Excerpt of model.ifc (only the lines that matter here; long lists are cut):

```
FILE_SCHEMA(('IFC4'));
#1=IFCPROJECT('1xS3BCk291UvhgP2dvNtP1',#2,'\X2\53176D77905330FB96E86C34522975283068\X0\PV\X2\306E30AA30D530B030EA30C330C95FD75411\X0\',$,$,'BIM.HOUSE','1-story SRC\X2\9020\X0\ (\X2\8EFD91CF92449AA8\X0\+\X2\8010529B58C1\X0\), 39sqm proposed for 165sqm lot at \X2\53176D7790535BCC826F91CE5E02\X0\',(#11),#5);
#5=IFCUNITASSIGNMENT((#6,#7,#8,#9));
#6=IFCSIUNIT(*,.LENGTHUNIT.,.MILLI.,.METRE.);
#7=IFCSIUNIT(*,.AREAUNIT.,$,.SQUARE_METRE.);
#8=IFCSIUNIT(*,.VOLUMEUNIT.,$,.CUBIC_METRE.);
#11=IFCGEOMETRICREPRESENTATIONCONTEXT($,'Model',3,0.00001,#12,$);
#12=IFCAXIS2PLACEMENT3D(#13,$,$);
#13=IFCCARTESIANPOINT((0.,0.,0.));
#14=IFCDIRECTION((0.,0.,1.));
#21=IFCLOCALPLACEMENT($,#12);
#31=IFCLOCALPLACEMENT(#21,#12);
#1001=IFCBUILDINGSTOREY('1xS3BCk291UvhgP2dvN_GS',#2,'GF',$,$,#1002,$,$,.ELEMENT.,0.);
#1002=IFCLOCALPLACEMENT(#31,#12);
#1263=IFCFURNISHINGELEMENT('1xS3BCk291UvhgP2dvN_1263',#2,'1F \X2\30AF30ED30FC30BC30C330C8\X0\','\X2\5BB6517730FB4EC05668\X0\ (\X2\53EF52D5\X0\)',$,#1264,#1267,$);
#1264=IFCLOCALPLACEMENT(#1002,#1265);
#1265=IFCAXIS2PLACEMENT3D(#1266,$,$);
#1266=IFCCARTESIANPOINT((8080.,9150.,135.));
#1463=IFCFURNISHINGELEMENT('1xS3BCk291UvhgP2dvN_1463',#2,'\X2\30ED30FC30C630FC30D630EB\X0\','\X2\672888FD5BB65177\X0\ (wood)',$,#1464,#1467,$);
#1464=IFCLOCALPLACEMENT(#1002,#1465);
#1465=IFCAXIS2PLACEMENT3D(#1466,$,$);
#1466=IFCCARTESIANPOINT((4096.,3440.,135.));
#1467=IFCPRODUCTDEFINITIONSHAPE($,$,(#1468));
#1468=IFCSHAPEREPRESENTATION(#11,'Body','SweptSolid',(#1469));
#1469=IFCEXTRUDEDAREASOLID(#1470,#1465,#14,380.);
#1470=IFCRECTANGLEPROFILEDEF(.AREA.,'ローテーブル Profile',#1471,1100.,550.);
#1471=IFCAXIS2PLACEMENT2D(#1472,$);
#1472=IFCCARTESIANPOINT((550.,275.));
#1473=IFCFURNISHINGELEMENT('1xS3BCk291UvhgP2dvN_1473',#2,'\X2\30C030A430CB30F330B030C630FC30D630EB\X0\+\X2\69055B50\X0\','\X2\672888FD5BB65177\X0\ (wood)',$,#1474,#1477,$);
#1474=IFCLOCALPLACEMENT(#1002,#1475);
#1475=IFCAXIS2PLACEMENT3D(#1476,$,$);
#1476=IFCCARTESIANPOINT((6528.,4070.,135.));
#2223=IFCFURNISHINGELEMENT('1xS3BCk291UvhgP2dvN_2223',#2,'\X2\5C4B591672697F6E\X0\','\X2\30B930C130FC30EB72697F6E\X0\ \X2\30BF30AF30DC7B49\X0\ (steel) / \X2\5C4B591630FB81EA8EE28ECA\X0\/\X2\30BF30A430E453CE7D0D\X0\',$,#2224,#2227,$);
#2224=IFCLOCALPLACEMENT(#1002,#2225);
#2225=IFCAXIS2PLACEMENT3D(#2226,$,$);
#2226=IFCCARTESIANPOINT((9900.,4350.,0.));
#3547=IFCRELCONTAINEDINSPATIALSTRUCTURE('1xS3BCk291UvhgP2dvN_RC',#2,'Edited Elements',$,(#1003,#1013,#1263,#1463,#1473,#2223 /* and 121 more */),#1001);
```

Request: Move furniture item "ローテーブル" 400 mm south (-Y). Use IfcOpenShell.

```python
import ifcopenshell
import ifcopenshell.api.geometry
import ifcopenshell.util.placement
import ifcopenshell.util.unit

model = ifcopenshell.open("model.ifc")
unit_scale = ifcopenshell.util.unit.calculate_unit_scale(model)

item = model.by_guid("1xS3BCk291UvhgP2dvN_1463")
matrix = ifcopenshell.util.placement.get_local_placement(item.ObjectPlacement)
matrix[1, 3] -= 0.4 / unit_scale
ifcopenshell.api.geometry.edit_object_placement(model, product=item, matrix=matrix, is_si=False)

print(ifcopenshell.util.placement.get_local_placement(item.ObjectPlacement).round(3) + 0.0)

model.write("model_rev.ifc")
```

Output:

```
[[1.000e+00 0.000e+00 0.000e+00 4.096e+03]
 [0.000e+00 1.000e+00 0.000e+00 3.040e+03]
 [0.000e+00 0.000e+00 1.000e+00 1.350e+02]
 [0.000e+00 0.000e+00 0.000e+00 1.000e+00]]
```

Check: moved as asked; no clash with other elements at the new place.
